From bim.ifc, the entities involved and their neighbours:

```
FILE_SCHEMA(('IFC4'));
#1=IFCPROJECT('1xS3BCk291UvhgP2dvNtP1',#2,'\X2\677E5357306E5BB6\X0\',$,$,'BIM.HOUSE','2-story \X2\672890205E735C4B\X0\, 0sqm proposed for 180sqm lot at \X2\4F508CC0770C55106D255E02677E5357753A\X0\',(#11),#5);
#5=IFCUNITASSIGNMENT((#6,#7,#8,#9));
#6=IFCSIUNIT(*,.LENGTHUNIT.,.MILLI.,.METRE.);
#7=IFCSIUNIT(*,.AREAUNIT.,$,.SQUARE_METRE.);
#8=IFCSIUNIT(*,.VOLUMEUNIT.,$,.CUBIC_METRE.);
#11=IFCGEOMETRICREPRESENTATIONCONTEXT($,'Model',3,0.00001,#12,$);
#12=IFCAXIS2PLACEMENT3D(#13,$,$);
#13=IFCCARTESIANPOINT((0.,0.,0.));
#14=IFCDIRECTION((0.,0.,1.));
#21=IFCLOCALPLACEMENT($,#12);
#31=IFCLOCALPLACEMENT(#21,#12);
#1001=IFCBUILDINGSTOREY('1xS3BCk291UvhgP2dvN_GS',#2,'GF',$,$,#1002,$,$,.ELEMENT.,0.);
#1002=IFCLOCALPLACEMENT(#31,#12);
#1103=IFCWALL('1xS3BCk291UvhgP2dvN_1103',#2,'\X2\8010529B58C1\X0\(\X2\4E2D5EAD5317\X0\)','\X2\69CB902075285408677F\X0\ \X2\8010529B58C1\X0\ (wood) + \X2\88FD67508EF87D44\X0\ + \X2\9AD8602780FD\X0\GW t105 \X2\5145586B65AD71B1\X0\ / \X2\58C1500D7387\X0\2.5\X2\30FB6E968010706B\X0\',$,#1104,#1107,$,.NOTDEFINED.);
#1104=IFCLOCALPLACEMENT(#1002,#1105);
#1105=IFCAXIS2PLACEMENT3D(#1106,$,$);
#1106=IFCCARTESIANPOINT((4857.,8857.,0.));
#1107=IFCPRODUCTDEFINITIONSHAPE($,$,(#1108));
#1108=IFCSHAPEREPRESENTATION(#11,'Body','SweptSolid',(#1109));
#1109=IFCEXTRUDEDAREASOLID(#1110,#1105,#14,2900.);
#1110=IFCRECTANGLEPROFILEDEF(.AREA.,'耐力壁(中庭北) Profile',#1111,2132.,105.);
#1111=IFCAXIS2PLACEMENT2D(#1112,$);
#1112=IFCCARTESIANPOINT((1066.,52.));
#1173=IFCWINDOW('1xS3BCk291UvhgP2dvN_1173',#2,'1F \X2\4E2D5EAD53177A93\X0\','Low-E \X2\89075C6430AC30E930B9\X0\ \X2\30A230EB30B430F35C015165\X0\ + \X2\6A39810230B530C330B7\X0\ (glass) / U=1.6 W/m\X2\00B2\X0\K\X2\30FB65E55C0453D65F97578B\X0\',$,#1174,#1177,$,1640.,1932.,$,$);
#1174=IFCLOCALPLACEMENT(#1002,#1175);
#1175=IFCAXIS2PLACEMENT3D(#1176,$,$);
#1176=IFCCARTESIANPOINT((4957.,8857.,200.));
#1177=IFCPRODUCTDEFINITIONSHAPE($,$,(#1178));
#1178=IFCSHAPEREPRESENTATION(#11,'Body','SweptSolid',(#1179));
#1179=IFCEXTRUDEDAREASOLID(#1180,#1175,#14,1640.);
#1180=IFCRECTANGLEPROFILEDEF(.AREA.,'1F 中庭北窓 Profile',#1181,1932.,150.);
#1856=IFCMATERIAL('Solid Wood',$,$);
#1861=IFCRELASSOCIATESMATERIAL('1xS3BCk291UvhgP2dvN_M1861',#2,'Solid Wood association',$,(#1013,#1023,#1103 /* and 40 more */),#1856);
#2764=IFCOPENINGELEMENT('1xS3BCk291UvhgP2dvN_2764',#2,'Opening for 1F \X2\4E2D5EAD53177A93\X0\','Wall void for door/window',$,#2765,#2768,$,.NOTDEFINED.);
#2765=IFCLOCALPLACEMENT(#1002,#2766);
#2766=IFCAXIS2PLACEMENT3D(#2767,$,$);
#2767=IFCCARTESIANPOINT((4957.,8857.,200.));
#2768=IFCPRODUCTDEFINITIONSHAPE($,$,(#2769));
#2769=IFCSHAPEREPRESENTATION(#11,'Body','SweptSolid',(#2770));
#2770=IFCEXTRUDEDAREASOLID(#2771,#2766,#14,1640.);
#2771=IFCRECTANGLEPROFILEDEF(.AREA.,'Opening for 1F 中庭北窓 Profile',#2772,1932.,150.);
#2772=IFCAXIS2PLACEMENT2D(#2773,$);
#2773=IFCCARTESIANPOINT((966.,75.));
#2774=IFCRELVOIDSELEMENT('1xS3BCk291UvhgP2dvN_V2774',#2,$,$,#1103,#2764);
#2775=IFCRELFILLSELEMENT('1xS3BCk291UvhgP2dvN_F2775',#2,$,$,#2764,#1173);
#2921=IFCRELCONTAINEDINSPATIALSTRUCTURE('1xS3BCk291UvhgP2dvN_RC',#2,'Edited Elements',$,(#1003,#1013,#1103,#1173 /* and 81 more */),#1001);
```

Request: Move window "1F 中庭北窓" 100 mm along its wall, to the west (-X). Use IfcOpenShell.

```python
import ifcopenshell
import ifcopenshell.api.geometry
import ifcopenshell.util.placement
import ifcopenshell.util.unit

model = ifcopenshell.open("bim.ifc")
unit_scale = ifcopenshell.util.unit.calculate_unit_scale(model)

window = model.by_guid("1xS3BCk291UvhgP2dvN_1173")
opening = window.FillsVoids[0].RelatingOpeningElement
wall = opening.VoidsElements[0].RelatingBuildingElement

wall_matrix = ifcopenshell.util.placement.get_local_placement(wall.ObjectPlacement)
shift = wall_matrix[:3, 0] * -0.1 / unit_scale
before = ifcopenshell.util.placement.get_local_placement(window.ObjectPlacement)[:3, 3].copy()

# The window is not placed relative to its opening, so move both.
for product in (opening, window):
    matrix = ifcopenshell.util.placement.get_local_placement(product.ObjectPlacement)
    matrix[:3, 3] += shift
    ifcopenshell.api.geometry.edit_object_placement(model, product=product, matrix=matrix, is_si=False)

after = ifcopenshell.util.placement.get_local_placement(window.ObjectPlacement)[:3, 3]
print("window moved by", (after - before).round(3) + 0.0)

model.write("bim_updated.ifc")
```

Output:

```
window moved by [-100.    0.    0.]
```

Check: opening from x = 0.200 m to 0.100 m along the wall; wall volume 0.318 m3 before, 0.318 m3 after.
